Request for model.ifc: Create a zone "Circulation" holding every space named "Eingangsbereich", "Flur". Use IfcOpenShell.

First a look at what the model holds.

```python
import ifcopenshell

model = ifcopenshell.open("model.ifc")
print(model.schema)
seen = {}
for space in model.by_type("IfcSpace"):
    seen[space.LongName] = seen.get(space.LongName, 0) + 1
for name, count in sorted(seen.items(), key=str):
    print(count, "x", name)
print("zones:", [z.Name for z in model.by_type("IfcZone")][:20])
```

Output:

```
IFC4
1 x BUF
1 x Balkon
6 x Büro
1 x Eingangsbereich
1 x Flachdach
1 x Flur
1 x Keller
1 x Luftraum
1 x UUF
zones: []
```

```python
import ifcopenshell
import ifcopenshell.api.group
import ifcopenshell.api.root

model = ifcopenshell.open("model.ifc")

names = {"Eingangsbereich", "Flur"}
spaces = [s for s in model.by_type("IfcSpace") if s.LongName in names]

zone = ifcopenshell.api.root.create_entity(model, ifc_class="IfcZone", name="Circulation")
ifcopenshell.api.group.assign_group(model, products=spaces, group=zone)
print(len(spaces), "spaces in", zone.Name)

model.write("model_updated.ifc")
```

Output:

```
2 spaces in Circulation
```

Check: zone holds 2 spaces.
